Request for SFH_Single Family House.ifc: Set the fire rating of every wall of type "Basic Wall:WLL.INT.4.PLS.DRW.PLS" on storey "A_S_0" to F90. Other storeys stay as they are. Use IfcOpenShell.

First a look at what the model holds.

```python
import ifcopenshell
import ifcopenshell.util.element

model = ifcopenshell.open("SFH_Single Family House.ifc")
print(model.schema)
storey = next(s for s in model.by_type("IfcBuildingStorey") if s.Name == "A_S_0")
walls = [e for e in ifcopenshell.util.element.get_decomposition(storey) if e.is_a("IfcWall")]
seen = {}
for e in walls:
    element_type = ifcopenshell.util.element.get_type(e)
    key = (element_type.Name if element_type != e and element_type else None, ifcopenshell.util.element.get_pset(e, "Pset_WallCommon", "FireRating"))
    seen[key] = seen.get(key, 0) + 1
for (name, value), count in sorted(seen.items(), key=str):
    print(count, "x", name, "|", value)
```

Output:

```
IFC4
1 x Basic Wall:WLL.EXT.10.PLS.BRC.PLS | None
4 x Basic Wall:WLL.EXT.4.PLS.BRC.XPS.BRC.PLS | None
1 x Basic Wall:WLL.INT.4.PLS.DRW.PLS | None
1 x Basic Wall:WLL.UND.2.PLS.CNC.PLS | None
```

```python
import ifcopenshell
import ifcopenshell.api.pset
import ifcopenshell.util.element

model = ifcopenshell.open("SFH_Single Family House.ifc")

storey = next(s for s in model.by_type("IfcBuildingStorey") if s.Name == "A_S_0")
walls = [e for e in ifcopenshell.util.element.get_decomposition(storey) if e.is_a("IfcWall")]

count = 0
for e in walls:
    element_type = ifcopenshell.util.element.get_type(e)
    if element_type in (None, e) or element_type.Name != "Basic Wall:WLL.INT.4.PLS.DRW.PLS":
        continue
    # add_pset returns the element's existing set when there is one.
    pset = ifcopenshell.api.pset.add_pset(model, product=e, name="Pset_WallCommon")
    ifcopenshell.api.pset.edit_pset(model, pset=pset, properties={"FireRating": "F90"})
    count += 1

print(count, "walls updated")

model.write("SFH_Single Family House_edited.ifc")
```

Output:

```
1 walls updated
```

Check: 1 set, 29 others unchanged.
